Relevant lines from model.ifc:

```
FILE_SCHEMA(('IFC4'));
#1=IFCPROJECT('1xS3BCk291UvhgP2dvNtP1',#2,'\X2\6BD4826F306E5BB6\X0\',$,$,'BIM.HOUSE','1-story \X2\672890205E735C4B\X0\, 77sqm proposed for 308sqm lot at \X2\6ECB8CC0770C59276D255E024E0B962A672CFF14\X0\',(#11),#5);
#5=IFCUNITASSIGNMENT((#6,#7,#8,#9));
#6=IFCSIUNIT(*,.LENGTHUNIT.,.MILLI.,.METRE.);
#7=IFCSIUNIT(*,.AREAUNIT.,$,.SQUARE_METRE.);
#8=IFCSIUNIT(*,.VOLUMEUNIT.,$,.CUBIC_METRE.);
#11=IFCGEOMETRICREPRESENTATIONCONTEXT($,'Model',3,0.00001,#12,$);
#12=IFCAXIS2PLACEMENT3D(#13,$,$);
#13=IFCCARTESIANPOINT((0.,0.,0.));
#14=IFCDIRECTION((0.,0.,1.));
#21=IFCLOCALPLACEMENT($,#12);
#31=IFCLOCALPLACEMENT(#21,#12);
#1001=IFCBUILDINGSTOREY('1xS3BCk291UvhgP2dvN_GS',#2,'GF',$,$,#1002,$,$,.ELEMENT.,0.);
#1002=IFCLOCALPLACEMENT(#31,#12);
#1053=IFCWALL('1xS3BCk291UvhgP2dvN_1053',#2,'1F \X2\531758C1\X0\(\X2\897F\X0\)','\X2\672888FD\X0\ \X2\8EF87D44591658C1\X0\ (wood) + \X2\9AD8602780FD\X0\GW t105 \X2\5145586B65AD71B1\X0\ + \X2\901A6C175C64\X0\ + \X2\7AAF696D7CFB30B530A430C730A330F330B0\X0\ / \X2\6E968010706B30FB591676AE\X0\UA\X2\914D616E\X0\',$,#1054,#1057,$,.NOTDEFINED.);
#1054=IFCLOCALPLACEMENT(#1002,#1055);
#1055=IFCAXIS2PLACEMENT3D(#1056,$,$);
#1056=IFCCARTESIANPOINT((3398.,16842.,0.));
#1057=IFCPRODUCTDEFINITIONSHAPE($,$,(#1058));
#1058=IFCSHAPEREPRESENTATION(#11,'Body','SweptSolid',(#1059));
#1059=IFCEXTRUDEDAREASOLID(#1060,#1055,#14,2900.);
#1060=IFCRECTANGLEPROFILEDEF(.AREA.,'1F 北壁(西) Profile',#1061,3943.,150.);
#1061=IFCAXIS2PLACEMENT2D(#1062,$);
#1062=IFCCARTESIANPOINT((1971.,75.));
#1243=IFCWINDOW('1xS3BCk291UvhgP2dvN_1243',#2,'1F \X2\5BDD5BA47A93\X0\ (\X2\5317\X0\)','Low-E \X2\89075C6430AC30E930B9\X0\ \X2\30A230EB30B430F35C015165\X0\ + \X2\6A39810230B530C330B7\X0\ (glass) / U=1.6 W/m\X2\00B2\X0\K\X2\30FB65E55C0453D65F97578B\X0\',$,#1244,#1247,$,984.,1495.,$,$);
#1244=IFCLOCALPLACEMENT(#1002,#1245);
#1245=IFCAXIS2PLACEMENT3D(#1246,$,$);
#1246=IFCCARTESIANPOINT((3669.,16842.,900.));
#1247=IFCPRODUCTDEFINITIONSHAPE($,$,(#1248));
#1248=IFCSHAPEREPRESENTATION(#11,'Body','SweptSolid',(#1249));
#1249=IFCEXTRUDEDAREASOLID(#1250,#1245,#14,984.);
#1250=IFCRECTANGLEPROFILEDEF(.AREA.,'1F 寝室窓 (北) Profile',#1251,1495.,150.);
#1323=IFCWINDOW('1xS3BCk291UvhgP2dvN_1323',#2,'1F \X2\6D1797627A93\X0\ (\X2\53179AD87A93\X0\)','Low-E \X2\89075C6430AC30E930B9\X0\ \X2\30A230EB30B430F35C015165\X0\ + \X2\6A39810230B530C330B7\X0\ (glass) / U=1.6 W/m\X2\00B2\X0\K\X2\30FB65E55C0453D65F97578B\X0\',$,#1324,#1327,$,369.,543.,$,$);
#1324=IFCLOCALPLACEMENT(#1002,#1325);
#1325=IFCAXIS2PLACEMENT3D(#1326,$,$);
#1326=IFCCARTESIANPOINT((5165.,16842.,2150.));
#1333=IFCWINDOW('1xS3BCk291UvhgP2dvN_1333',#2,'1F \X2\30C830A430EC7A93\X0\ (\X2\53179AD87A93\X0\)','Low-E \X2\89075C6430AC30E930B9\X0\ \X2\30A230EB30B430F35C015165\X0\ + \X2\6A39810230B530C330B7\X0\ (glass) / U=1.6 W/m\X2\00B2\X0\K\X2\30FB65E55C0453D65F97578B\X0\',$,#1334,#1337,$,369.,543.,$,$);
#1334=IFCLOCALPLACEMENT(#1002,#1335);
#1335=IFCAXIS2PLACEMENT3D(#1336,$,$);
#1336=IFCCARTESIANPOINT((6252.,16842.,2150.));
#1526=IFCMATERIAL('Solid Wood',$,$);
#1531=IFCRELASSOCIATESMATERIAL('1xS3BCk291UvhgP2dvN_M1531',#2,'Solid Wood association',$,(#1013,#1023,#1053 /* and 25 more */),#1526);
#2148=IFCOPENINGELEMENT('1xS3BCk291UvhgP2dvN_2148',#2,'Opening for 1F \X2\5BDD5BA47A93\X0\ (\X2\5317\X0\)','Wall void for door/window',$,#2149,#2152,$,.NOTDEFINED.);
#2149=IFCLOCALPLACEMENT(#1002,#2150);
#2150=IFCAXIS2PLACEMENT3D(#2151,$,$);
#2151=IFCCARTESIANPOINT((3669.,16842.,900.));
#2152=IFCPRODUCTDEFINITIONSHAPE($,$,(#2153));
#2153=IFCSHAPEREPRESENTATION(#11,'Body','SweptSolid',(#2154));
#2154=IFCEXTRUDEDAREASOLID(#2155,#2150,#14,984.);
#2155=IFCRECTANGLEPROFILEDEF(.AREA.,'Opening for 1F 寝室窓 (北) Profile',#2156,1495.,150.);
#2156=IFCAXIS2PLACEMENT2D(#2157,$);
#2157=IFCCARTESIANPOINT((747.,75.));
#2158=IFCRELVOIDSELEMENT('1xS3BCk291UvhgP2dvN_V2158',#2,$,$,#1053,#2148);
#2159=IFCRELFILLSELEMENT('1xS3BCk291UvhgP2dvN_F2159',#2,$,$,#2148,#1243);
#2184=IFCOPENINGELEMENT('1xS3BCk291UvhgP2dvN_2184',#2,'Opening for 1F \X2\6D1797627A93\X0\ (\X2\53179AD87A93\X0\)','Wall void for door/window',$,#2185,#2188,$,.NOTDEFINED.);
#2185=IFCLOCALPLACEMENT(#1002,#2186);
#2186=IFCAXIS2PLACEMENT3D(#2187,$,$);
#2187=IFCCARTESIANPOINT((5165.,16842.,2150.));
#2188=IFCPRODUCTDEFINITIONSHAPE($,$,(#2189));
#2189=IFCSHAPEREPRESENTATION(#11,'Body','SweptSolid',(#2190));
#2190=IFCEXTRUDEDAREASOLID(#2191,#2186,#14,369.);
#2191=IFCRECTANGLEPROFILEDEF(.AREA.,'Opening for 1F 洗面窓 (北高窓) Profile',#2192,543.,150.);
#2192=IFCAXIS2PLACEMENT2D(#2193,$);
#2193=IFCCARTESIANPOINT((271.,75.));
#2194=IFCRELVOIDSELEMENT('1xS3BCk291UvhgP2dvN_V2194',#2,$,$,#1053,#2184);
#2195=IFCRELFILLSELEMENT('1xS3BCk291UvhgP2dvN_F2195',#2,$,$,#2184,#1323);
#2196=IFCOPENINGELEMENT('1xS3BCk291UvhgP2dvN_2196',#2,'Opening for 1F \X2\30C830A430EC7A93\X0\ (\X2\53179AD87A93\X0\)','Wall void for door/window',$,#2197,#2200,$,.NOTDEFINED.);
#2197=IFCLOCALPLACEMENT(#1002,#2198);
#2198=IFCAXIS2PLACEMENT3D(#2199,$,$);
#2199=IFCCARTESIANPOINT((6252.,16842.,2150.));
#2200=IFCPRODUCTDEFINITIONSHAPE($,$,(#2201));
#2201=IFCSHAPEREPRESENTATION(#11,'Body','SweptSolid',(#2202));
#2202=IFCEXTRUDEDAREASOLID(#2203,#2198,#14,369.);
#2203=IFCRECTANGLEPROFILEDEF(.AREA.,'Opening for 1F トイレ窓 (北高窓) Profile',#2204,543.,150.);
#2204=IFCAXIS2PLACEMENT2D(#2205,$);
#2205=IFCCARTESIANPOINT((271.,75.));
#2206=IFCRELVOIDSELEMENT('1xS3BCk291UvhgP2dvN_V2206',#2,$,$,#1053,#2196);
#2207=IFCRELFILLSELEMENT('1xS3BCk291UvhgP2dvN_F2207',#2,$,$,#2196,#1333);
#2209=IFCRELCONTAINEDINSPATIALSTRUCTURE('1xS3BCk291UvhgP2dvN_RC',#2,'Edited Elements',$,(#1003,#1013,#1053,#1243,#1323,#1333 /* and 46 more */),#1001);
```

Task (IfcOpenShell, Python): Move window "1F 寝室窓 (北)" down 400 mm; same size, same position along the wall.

```python
import numpy as np
import ifcopenshell
import ifcopenshell.api.geometry
import ifcopenshell.util.placement
import ifcopenshell.util.unit

model = ifcopenshell.open("model.ifc")
unit_scale = ifcopenshell.util.unit.calculate_unit_scale(model)

window = model.by_id(1243)
opening = window.FillsVoids[0].RelatingOpeningElement
dz = -0.4 / unit_scale

shift = np.array([0.0, 0.0, dz])
# The window is not placed relative to its opening, so move both.
for product in (opening, window):
    matrix = ifcopenshell.util.placement.get_local_placement(product.ObjectPlacement)
    matrix[:3, 3] += shift
    ifcopenshell.api.geometry.edit_object_placement(model, product=product, matrix=matrix, is_si=False)

print(f"moved by {dz * unit_scale:+.3f} m")

model.write("model_rev.ifc")
```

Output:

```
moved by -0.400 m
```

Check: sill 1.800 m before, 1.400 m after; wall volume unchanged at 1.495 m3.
